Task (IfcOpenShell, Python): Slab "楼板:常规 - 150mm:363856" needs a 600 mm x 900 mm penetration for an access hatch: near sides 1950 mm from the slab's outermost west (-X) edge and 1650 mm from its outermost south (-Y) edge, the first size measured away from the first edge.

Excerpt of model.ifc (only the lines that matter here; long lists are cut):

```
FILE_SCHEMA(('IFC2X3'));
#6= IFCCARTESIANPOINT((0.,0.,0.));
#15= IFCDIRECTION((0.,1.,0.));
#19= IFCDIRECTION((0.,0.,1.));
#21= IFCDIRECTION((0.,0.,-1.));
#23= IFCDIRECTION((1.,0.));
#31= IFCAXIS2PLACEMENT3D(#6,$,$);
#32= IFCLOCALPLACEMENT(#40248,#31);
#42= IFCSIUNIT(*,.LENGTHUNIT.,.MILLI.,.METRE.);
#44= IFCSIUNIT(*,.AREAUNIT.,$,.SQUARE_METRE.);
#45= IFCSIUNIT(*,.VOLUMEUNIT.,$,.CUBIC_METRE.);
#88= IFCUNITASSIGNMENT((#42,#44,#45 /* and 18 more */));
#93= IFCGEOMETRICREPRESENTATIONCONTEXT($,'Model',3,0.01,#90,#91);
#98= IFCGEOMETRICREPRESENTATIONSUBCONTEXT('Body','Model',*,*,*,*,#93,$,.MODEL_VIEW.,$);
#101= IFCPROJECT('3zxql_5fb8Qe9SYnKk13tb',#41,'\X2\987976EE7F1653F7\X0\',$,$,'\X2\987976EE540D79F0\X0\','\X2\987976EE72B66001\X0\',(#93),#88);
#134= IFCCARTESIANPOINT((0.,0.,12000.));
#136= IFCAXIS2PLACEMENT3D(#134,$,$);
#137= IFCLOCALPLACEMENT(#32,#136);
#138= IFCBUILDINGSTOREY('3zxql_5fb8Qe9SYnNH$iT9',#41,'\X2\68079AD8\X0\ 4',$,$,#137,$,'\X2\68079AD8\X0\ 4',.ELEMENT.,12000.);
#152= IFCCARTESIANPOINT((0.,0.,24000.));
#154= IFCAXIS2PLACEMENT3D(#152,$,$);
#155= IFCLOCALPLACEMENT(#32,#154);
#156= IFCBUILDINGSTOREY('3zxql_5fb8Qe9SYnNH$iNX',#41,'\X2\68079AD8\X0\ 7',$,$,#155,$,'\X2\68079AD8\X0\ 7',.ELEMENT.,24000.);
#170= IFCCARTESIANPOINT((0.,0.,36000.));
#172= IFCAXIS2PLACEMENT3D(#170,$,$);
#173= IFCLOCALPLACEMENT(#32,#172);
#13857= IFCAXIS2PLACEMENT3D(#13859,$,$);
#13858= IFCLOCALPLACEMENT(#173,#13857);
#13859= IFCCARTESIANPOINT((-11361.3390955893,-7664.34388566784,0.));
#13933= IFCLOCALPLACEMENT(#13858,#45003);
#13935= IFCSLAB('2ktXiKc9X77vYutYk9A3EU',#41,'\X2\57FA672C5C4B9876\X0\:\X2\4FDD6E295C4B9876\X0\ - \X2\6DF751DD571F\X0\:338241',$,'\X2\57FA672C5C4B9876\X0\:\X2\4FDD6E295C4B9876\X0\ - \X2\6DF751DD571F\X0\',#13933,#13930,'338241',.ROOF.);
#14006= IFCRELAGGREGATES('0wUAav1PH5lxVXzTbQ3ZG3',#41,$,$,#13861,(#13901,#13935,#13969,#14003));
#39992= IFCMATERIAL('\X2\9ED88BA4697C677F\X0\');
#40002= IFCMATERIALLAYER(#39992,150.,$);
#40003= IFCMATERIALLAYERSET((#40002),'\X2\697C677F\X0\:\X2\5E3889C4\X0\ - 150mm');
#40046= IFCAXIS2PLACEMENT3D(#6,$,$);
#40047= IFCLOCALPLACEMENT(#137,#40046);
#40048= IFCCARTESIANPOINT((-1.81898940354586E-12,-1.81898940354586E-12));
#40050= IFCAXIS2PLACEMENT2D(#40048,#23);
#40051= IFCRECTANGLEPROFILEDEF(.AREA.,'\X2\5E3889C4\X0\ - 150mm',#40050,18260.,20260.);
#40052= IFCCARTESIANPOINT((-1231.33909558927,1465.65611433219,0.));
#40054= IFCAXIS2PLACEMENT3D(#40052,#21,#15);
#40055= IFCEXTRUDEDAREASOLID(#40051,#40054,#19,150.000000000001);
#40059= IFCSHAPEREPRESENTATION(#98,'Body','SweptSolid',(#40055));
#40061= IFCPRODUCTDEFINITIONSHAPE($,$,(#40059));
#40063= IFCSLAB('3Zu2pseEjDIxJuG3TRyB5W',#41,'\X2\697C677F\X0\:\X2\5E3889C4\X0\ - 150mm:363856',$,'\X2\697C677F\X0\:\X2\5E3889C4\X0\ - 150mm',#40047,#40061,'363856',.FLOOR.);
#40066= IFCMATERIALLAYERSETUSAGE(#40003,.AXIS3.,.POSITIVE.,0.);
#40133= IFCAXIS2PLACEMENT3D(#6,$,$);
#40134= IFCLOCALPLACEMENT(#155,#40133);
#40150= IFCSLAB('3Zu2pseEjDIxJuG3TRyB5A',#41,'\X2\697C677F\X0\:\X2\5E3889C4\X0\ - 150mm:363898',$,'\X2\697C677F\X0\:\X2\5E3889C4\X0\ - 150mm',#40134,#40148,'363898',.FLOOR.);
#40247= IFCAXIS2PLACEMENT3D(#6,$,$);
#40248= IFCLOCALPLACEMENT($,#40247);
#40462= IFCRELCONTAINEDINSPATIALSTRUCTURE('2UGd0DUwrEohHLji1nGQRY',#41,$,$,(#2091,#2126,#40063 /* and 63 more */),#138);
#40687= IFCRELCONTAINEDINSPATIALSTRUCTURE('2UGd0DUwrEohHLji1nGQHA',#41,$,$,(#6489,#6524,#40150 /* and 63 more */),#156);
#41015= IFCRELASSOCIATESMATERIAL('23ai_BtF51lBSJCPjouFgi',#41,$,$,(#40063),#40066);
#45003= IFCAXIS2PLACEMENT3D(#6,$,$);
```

```python
import numpy as np
import ifcopenshell
import ifcopenshell.api.feature
import ifcopenshell.api.geometry
import ifcopenshell.api.root
import ifcopenshell.geom
import ifcopenshell.util.placement
import ifcopenshell.util.representation
import ifcopenshell.util.shape
import ifcopenshell.util.unit

model = ifcopenshell.open("model.ifc")
unit_scale = ifcopenshell.util.unit.calculate_unit_scale(model)
settings = ifcopenshell.geom.settings()


def volume(element):
    """Net volume in cubic metres, openings subtracted."""
    shape = ifcopenshell.geom.create_shape(settings, element)
    return ifcopenshell.util.shape.get_volume(shape.geometry)


slab = model.by_id(40063)
before = volume(slab)

# Extent in the slab's own axes, in metres. The edges named are its -X and -Y sides.
slab_shape = ifcopenshell.geom.create_shape(settings, slab)
vertices = ifcopenshell.util.shape.get_vertices(slab_shape.geometry)
x_min, y_min, bottom = vertices.min(axis=0)
top = vertices[:, 2].max()

opening = ifcopenshell.api.root.create_entity(model, ifc_class="IfcOpeningElement", name="Access hatch opening")
context = ifcopenshell.util.representation.get_context(model, "Model", "Body", "MODEL_VIEW")
width, depth = 0.6, 0.9
outline = [(0.0, 0.0), (width, 0.0), (width, depth), (0.0, depth), (0.0, 0.0)]
# Overshoot both faces by 50 mm so the cut is clean.
shape = ifcopenshell.api.geometry.add_slab_representation(
    model, context=context, depth=top - bottom + 0.1, polyline=outline
)
ifcopenshell.api.geometry.assign_representation(model, product=opening, representation=shape)

matrix = ifcopenshell.util.placement.get_local_placement(slab.ObjectPlacement)
matrix[:, 3] = matrix @ np.append(np.array([x_min + 1.95, y_min + 1.65, bottom - 0.05]) / unit_scale, 1.0)
ifcopenshell.api.geometry.edit_object_placement(model, product=opening, matrix=matrix, is_si=False)
ifcopenshell.api.feature.add_feature(model, feature=opening, element=slab)

after = volume(slab)

print(f"slab volume {before:.3f} -> {after:.3f} m3")

model.write("model-out.ifc")
```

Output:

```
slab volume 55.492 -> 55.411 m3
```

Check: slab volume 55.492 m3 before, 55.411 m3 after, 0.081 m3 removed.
